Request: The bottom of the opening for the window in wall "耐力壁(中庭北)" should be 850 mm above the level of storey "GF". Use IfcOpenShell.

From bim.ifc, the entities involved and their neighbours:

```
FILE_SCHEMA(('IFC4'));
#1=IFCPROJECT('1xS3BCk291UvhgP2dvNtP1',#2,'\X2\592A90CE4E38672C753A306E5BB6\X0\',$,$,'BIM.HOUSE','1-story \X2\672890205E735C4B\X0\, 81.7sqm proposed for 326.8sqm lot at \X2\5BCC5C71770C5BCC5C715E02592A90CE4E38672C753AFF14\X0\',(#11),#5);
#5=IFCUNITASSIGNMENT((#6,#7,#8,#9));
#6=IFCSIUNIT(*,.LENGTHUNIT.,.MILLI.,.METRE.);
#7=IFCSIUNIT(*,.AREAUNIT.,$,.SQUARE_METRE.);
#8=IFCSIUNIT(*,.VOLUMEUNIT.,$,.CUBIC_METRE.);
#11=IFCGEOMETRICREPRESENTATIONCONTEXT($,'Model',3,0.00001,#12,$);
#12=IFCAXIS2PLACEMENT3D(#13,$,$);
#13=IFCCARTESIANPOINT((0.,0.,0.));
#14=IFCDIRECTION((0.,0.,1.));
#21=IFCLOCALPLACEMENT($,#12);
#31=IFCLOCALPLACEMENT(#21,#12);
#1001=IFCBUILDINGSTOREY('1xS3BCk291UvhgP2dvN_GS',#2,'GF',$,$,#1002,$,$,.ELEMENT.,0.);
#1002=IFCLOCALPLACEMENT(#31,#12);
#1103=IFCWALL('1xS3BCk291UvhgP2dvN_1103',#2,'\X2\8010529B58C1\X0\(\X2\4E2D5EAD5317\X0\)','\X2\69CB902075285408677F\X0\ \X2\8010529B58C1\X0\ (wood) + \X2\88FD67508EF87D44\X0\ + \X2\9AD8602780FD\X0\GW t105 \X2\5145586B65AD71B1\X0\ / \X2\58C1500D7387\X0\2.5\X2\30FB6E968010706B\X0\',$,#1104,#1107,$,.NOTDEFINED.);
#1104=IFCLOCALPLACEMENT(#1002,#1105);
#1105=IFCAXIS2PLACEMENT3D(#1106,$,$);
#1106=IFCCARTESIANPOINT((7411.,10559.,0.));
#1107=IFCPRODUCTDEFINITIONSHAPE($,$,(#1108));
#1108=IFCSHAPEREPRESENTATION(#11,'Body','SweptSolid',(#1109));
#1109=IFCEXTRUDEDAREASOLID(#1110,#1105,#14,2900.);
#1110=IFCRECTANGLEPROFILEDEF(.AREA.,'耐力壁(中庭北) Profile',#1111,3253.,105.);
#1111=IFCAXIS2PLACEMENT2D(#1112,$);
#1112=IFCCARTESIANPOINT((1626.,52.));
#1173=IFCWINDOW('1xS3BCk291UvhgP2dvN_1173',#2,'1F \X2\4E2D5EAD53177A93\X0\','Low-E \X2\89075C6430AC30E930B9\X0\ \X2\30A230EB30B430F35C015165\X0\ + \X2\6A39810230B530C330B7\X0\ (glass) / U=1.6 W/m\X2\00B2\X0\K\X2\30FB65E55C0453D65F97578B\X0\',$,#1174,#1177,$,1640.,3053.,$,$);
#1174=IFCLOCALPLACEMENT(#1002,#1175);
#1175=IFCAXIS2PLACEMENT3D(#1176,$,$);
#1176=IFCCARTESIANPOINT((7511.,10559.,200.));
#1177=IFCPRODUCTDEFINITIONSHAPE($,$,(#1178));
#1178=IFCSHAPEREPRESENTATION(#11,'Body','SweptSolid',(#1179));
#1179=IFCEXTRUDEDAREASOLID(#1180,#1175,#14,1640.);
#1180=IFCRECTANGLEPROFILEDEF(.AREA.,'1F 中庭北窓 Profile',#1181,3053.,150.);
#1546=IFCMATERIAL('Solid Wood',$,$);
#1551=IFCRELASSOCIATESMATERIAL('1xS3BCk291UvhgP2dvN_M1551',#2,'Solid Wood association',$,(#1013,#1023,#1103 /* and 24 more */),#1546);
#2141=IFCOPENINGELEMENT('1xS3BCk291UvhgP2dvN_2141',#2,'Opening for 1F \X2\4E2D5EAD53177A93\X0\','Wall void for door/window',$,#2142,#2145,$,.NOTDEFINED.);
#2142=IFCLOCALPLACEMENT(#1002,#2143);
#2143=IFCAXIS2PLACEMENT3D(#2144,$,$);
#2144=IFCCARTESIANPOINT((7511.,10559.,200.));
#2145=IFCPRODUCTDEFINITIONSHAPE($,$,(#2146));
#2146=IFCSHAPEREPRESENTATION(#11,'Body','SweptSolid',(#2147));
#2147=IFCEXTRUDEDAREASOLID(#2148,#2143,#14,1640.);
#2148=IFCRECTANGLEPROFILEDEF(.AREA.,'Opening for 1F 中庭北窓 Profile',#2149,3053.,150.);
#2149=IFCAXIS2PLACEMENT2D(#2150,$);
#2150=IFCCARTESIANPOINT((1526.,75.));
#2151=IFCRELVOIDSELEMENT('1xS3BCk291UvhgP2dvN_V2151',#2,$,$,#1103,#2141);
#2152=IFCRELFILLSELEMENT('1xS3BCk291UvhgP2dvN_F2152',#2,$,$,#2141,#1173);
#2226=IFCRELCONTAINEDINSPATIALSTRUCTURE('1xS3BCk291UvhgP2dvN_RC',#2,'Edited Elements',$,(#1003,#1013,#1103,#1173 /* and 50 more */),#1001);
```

```python
import numpy as np
import ifcopenshell
import ifcopenshell.api.geometry
import ifcopenshell.geom
import ifcopenshell.util.element
import ifcopenshell.util.placement
import ifcopenshell.util.shape
import ifcopenshell.util.unit

model = ifcopenshell.open("bim.ifc")
unit_scale = ifcopenshell.util.unit.calculate_unit_scale(model)

window = model.by_guid("1xS3BCk291UvhgP2dvN_1173")
opening = window.FillsVoids[0].RelatingOpeningElement
storey = ifcopenshell.util.element.get_container(window, ifc_class="IfcBuildingStorey")
level = ifcopenshell.util.placement.get_local_placement(storey.ObjectPlacement)[2, 3]

# The opening's origin need not be at the sill, so measure its lowest point.
shape = ifcopenshell.geom.create_shape(ifcopenshell.geom.settings(), opening)
bottom = ifcopenshell.util.shape.get_shape_bottom_elevation(shape, shape.geometry) / unit_scale
dz = level + 0.85 / unit_scale - bottom

shift = np.array([0.0, 0.0, dz])
# The window is not placed relative to its opening, so move both.
for product in (opening, window):
    matrix = ifcopenshell.util.placement.get_local_placement(product.ObjectPlacement)
    matrix[:3, 3] += shift
    ifcopenshell.api.geometry.edit_object_placement(model, product=product, matrix=matrix, is_si=False)

print(f"moved by {dz * unit_scale:+.3f} m")

model.write("bim_edited.ifc")
```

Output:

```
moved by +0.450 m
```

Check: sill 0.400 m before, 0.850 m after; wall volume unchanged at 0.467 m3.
